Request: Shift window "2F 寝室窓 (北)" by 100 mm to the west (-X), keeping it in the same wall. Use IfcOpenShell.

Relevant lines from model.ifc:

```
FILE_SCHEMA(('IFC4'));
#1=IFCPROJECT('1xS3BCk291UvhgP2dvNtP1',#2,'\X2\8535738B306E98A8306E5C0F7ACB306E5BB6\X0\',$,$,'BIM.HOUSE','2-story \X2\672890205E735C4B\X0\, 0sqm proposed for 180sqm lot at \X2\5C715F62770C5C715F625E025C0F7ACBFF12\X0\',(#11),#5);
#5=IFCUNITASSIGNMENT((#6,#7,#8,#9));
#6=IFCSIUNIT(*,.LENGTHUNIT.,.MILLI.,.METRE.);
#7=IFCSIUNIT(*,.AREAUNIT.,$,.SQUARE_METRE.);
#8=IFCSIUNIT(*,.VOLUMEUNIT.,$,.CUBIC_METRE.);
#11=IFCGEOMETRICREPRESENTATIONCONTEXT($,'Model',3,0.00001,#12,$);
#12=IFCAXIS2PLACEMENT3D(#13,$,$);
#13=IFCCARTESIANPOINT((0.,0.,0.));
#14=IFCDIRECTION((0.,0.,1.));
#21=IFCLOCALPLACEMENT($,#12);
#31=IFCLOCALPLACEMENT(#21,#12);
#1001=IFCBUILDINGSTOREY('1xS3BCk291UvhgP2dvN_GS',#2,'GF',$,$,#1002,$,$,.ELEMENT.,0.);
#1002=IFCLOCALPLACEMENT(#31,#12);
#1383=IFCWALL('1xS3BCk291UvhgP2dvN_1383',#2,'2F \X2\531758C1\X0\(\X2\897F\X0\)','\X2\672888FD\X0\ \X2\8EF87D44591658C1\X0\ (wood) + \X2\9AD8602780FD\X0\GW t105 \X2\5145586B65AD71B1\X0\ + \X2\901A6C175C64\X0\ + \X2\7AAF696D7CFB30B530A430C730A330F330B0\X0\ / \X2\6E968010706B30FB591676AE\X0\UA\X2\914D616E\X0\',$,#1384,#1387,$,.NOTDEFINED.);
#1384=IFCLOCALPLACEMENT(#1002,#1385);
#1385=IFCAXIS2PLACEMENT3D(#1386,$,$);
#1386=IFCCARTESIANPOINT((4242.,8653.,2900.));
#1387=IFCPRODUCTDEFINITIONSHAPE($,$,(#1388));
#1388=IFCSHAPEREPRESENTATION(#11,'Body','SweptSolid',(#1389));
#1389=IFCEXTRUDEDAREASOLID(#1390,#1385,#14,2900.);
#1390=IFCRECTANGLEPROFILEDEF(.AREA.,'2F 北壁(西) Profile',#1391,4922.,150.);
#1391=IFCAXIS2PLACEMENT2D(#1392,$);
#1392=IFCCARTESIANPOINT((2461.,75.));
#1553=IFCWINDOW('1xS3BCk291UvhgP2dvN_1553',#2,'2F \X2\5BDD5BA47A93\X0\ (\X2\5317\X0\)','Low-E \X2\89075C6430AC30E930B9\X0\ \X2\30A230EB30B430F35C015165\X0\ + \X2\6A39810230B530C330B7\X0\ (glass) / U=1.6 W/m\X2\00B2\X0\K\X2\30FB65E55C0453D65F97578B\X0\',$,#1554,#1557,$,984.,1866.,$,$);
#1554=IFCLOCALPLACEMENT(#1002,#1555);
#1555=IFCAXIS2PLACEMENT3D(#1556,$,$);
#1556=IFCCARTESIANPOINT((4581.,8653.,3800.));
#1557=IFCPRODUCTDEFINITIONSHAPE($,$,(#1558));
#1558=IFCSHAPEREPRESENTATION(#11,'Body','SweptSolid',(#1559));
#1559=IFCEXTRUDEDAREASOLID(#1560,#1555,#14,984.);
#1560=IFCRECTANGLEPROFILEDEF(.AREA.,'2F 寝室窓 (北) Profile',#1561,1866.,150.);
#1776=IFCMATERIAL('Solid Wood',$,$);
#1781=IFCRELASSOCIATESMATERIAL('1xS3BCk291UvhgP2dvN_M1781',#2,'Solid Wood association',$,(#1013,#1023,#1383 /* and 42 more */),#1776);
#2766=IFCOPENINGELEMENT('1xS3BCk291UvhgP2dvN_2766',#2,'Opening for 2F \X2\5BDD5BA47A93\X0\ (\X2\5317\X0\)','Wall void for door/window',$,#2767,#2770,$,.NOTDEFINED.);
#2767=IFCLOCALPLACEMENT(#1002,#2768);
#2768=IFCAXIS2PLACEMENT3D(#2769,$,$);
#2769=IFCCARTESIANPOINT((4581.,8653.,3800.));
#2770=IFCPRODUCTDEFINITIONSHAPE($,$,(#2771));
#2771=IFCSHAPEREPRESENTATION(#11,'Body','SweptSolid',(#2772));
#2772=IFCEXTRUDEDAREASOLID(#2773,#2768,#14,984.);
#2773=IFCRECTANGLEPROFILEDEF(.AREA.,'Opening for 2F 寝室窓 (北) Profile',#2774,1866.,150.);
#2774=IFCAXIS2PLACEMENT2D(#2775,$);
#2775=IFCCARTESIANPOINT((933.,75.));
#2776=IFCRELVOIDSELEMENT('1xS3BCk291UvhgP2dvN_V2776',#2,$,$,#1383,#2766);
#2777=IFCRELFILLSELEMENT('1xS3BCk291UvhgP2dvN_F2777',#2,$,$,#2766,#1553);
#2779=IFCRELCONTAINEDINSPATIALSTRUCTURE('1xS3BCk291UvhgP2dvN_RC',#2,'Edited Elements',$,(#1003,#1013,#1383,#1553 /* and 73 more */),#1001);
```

```python
import ifcopenshell
import ifcopenshell.api.geometry
import ifcopenshell.util.placement
import ifcopenshell.util.unit

model = ifcopenshell.open("model.ifc")
unit_scale = ifcopenshell.util.unit.calculate_unit_scale(model)

window = model.by_guid("1xS3BCk291UvhgP2dvN_1553")
opening = window.FillsVoids[0].RelatingOpeningElement
wall = opening.VoidsElements[0].RelatingBuildingElement

wall_matrix = ifcopenshell.util.placement.get_local_placement(wall.ObjectPlacement)
shift = wall_matrix[:3, 0] * -0.1 / unit_scale
before = ifcopenshell.util.placement.get_local_placement(window.ObjectPlacement)[:3, 3].copy()

# The window is not placed relative to its opening, so move both.
for product in (opening, window):
    matrix = ifcopenshell.util.placement.get_local_placement(product.ObjectPlacement)
    matrix[:3, 3] += shift
    ifcopenshell.api.geometry.edit_object_placement(model, product=product, matrix=matrix, is_si=False)

after = ifcopenshell.util.placement.get_local_placement(window.ObjectPlacement)[:3, 3]
print("window moved by", (after - before).round(3) + 0.0)

model.write("model_v2.ifc")
```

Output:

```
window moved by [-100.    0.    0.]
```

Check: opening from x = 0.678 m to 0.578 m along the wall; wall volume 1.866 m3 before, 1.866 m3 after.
